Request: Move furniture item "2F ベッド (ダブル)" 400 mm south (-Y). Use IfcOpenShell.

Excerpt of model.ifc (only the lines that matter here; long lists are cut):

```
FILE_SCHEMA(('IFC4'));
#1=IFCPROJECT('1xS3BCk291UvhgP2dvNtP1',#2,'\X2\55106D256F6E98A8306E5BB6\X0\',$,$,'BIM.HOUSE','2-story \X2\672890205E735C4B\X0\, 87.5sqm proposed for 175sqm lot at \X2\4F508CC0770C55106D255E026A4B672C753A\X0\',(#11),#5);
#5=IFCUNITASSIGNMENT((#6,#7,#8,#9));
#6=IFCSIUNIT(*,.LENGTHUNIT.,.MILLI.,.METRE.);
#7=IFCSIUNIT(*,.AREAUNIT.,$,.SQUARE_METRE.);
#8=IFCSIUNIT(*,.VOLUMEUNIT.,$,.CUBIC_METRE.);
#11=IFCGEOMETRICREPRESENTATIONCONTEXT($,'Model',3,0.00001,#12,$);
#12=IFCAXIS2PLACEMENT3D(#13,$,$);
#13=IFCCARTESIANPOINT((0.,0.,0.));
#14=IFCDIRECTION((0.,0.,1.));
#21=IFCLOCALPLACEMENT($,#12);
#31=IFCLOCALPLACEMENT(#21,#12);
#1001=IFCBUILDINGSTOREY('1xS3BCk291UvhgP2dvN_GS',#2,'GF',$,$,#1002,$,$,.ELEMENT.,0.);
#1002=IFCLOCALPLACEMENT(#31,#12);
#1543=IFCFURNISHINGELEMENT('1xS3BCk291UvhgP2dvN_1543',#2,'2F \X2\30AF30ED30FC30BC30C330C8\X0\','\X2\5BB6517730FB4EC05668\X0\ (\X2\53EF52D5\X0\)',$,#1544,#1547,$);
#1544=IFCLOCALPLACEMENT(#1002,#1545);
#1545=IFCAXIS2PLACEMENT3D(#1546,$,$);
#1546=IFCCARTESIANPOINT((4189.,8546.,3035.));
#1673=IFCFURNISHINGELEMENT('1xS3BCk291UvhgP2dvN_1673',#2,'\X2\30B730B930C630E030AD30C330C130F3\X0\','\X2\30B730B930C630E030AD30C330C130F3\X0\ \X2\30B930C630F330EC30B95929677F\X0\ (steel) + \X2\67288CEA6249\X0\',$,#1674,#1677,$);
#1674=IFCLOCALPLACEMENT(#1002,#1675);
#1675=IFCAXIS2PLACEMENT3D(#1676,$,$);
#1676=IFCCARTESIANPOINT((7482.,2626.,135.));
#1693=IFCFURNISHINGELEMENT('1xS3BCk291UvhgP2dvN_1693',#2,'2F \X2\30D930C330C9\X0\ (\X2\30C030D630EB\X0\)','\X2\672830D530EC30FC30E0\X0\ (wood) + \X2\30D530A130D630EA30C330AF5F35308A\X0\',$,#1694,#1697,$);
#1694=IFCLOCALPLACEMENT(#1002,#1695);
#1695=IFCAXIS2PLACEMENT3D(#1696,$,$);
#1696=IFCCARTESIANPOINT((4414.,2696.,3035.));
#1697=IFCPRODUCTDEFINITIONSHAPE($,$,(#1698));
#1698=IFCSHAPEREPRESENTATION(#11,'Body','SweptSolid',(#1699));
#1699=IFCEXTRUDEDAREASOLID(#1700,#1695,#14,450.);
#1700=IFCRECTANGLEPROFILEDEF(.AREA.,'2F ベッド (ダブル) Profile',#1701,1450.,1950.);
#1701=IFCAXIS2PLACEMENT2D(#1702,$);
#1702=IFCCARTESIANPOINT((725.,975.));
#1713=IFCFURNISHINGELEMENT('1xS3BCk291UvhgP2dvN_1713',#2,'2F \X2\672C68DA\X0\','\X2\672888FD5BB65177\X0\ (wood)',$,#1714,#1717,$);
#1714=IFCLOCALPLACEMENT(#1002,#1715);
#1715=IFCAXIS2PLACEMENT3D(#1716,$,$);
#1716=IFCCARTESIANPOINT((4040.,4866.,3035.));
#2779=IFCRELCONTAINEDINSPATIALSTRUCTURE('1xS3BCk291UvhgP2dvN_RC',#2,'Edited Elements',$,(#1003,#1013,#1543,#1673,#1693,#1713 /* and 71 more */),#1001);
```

```python
import ifcopenshell
import ifcopenshell.api.geometry
import ifcopenshell.util.placement

model = ifcopenshell.open("model.ifc")

item = model.by_guid("1xS3BCk291UvhgP2dvN_1693")
matrix = ifcopenshell.util.placement.get_local_placement(item.ObjectPlacement)
matrix[1, 3] -= 400.0
ifcopenshell.api.geometry.edit_object_placement(model, product=item, matrix=matrix, is_si=False)

print(ifcopenshell.util.placement.get_local_placement(item.ObjectPlacement).round(3) + 0.0)

model.write("model_updated.ifc")
```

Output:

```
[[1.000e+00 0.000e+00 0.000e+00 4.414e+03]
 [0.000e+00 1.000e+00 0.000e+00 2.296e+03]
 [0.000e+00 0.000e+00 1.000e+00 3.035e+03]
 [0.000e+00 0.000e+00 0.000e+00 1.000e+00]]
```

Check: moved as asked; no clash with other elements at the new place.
